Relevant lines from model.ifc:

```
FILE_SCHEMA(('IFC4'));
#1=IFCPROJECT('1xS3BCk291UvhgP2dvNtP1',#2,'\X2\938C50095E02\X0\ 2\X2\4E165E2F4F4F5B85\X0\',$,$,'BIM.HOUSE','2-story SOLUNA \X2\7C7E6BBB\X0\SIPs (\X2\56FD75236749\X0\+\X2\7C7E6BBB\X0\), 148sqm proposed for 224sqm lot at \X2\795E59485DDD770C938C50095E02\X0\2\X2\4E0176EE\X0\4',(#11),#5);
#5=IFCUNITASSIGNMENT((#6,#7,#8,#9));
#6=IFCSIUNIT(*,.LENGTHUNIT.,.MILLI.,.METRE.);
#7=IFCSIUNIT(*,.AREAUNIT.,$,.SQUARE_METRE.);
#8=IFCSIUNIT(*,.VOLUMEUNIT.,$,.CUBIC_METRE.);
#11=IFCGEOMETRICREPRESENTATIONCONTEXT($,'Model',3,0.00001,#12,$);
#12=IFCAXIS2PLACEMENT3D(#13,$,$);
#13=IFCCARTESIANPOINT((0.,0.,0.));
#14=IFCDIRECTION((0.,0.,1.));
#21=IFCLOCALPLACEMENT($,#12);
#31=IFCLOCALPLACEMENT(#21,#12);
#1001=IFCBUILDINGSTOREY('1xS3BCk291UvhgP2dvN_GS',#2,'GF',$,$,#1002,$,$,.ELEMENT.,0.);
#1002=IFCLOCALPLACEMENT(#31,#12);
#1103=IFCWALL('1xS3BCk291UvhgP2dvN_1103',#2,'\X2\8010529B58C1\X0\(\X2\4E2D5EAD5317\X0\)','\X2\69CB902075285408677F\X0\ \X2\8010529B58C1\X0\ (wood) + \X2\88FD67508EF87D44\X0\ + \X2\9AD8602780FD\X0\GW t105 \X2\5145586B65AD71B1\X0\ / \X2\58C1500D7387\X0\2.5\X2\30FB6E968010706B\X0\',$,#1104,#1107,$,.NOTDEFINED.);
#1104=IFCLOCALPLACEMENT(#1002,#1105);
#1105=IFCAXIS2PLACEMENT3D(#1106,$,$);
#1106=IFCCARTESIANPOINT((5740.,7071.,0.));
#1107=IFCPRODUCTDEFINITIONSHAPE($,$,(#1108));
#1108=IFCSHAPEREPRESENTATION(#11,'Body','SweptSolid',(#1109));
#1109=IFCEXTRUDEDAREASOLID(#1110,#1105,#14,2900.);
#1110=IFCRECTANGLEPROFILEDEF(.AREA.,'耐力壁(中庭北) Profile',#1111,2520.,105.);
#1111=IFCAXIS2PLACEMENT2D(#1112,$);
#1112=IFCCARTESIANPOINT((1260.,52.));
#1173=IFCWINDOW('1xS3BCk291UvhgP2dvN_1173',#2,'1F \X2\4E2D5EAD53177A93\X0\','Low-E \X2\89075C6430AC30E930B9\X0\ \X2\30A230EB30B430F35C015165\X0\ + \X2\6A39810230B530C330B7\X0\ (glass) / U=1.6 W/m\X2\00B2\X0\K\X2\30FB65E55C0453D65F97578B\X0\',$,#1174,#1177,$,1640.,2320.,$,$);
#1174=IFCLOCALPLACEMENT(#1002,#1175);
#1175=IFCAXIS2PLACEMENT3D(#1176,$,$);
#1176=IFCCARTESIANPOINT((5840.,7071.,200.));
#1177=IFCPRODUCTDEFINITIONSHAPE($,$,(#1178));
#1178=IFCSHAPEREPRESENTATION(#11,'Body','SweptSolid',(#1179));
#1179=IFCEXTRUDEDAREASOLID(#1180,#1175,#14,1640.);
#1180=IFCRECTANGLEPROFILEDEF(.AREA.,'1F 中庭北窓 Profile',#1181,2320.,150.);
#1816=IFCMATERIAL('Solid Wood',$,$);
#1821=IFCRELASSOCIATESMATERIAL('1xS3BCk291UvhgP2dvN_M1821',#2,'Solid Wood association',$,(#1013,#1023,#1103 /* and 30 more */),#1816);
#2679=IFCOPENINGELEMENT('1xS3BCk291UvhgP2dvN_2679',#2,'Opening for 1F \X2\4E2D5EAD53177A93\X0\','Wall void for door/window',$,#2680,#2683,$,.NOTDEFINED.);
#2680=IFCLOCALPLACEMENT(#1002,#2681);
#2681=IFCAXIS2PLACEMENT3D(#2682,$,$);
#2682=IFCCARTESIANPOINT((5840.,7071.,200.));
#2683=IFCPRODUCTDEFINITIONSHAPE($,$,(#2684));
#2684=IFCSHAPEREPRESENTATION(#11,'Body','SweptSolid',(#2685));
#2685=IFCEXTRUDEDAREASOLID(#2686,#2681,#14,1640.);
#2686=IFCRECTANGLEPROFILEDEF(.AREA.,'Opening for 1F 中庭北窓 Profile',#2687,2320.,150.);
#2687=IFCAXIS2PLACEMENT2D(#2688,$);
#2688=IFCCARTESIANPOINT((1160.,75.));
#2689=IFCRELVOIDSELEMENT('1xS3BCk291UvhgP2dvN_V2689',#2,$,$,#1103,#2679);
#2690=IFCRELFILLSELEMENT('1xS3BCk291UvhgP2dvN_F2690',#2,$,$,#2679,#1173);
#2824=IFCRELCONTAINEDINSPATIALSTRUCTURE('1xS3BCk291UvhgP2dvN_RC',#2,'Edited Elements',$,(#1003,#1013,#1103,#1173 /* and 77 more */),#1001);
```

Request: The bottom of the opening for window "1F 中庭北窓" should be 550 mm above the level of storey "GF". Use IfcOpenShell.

```python
import numpy as np
import ifcopenshell
import ifcopenshell.api.geometry
import ifcopenshell.geom
import ifcopenshell.util.element
import ifcopenshell.util.placement
import ifcopenshell.util.shape
import ifcopenshell.util.unit

model = ifcopenshell.open("model.ifc")
unit_scale = ifcopenshell.util.unit.calculate_unit_scale(model)

window = model.by_guid("1xS3BCk291UvhgP2dvN_1173")
opening = window.FillsVoids[0].RelatingOpeningElement
storey = ifcopenshell.util.element.get_container(window, ifc_class="IfcBuildingStorey")
level = ifcopenshell.util.placement.get_local_placement(storey.ObjectPlacement)[2, 3]

# The opening's origin need not be at the sill, so measure its lowest point.
shape = ifcopenshell.geom.create_shape(ifcopenshell.geom.settings(), opening)
bottom = ifcopenshell.util.shape.get_shape_bottom_elevation(shape, shape.geometry) / unit_scale
dz = level + 550.0 - bottom

shift = np.array([0.0, 0.0, dz])
# The window is not placed relative to its opening, so move both.
for product in (opening, window):
    matrix = ifcopenshell.util.placement.get_local_placement(product.ObjectPlacement)
    matrix[:3, 3] += shift
    ifcopenshell.api.geometry.edit_object_placement(model, product=product, matrix=matrix, is_si=False)

print(f"moved by {dz * unit_scale:+.3f} m")

model.write("model_rev.ifc")
```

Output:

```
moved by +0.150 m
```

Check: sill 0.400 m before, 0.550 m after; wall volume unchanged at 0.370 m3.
